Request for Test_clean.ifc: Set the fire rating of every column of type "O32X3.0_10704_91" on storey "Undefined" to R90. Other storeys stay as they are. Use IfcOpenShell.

First a look at what the model holds.

```python
import ifcopenshell
import ifcopenshell.util.element

model = ifcopenshell.open("Test_clean.ifc")
print(model.schema)
storey = next(s for s in model.by_type("IfcBuildingStorey") if s.Name == "Undefined")
columns = [e for e in ifcopenshell.util.element.get_decomposition(storey) if e.is_a("IfcColumn")]
seen = {}
for e in columns:
    element_type = ifcopenshell.util.element.get_type(e)
    key = (element_type.Name if element_type != e and element_type else None, ifcopenshell.util.element.get_pset(e, "Pset_ColumnCommon", "FireRating"))
    seen[key] = seen.get(key, 0) + 1
for (name, value), count in sorted(seen.items(), key=str):
    print(count, "x", name, "|", value)
```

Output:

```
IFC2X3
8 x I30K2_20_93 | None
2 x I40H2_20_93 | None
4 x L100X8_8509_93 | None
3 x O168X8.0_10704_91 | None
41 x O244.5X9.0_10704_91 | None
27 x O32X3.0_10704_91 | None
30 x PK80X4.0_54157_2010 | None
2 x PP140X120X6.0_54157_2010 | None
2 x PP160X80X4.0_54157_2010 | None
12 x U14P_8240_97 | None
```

```python
import ifcopenshell
import ifcopenshell.api.pset
import ifcopenshell.util.element

model = ifcopenshell.open("Test_clean.ifc")

storey = next(s for s in model.by_type("IfcBuildingStorey") if s.Name == "Undefined")
columns = [e for e in ifcopenshell.util.element.get_decomposition(storey) if e.is_a("IfcColumn")]

count = 0
for e in columns:
    element_type = ifcopenshell.util.element.get_type(e)
    if element_type in (None, e) or element_type.Name != "O32X3.0_10704_91":
        continue
    found = ifcopenshell.util.element.get_pset(e, "Pset_ColumnCommon", should_inherit=False)
    if found:
        pset = model.by_id(found["id"])
        if len(ifcopenshell.util.element.get_elements_by_pset(pset)) > 1:
            pset = ifcopenshell.api.pset.unshare_pset(model, products=[e], pset=pset)[0]
    else:
        pset = ifcopenshell.api.pset.add_pset(model, product=e, name="Pset_ColumnCommon")
    ifcopenshell.api.pset.edit_pset(model, pset=pset, properties={"FireRating": "R90"})
    count += 1

print(count, "columns updated")

model.write("Test_clean_edited.ifc")
```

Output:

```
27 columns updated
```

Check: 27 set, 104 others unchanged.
